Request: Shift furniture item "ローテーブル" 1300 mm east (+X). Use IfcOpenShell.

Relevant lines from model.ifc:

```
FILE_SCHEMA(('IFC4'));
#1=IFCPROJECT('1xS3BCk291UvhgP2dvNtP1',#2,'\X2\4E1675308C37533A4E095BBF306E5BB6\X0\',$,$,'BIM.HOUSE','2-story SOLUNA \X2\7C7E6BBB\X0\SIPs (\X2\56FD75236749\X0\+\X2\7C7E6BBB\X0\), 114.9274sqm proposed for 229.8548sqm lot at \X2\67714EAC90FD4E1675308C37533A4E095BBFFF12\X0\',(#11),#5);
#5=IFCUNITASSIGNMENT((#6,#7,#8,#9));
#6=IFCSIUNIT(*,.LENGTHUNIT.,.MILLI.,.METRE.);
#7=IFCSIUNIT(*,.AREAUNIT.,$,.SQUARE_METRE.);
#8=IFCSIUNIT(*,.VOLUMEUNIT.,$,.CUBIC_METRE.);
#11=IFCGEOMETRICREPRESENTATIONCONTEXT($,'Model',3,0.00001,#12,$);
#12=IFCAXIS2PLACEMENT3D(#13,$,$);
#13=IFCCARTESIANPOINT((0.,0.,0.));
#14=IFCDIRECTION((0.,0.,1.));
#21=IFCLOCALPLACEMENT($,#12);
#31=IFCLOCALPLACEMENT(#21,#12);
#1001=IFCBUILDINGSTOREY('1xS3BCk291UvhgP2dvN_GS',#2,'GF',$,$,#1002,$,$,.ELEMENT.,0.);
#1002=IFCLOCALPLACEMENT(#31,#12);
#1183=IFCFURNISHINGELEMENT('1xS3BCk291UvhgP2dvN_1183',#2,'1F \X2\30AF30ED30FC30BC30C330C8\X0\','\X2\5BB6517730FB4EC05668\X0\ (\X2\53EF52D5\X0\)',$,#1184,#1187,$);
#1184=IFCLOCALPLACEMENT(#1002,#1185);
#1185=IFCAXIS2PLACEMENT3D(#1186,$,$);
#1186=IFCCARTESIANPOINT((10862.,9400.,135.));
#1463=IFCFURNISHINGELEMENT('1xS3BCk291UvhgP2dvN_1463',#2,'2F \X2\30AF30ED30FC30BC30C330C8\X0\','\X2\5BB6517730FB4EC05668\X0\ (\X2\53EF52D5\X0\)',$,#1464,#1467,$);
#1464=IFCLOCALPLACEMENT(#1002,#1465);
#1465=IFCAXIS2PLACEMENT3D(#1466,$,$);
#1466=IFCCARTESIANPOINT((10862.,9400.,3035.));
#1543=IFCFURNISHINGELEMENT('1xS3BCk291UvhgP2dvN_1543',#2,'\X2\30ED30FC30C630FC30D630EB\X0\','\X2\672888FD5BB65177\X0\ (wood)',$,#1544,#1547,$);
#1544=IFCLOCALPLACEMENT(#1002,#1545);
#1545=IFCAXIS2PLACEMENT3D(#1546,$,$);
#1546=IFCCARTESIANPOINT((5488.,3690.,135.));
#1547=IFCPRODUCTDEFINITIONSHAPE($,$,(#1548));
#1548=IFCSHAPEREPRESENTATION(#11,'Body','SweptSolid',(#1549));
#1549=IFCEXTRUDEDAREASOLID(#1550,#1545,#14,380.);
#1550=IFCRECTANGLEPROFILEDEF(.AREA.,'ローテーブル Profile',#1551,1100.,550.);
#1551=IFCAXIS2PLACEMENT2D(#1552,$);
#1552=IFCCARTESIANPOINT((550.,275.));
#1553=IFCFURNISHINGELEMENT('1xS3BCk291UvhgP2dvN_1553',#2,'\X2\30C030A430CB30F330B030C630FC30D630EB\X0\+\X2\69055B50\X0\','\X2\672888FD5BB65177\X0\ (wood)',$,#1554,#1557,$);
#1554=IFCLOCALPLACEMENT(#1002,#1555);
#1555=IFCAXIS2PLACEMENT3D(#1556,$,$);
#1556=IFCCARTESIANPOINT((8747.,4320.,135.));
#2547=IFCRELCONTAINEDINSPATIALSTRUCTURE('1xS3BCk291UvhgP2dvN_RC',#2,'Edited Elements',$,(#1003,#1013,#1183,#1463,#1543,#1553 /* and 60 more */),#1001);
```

```python
import ifcopenshell
import ifcopenshell.api.geometry
import ifcopenshell.util.placement
import ifcopenshell.util.unit

model = ifcopenshell.open("model.ifc")
unit_scale = ifcopenshell.util.unit.calculate_unit_scale(model)

item = model.by_guid("1xS3BCk291UvhgP2dvN_1543")
matrix = ifcopenshell.util.placement.get_local_placement(item.ObjectPlacement)
matrix[0, 3] += 1.3 / unit_scale
ifcopenshell.api.geometry.edit_object_placement(model, product=item, matrix=matrix, is_si=False)

print(ifcopenshell.util.placement.get_local_placement(item.ObjectPlacement).round(3) + 0.0)

model.write("model-out.ifc")
```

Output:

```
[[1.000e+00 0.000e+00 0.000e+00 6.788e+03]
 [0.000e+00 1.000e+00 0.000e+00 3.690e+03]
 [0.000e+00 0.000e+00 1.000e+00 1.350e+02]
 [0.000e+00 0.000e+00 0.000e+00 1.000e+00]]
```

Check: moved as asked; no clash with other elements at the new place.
